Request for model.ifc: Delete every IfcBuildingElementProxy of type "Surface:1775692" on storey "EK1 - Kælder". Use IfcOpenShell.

First a look at what the model holds.

```python
import ifcopenshell
import ifcopenshell.util.element

model = ifcopenshell.open("model.ifc")
print(model.schema)
storey = next(s for s in model.by_type("IfcBuildingStorey") if s.Name == "EK1 - Kælder")
proxies = [e for e in ifcopenshell.util.element.get_decomposition(storey) if e.is_a("IfcBuildingElementProxy")]
seen = {}
for e in proxies:
    element_type = ifcopenshell.util.element.get_type(e)
    name = element_type.Name if element_type not in (None, e) else None
    seen[name] = seen.get(name, 0) + 1
for name, count in sorted(seen.items(), key=str):
    print(count, "x", name)
```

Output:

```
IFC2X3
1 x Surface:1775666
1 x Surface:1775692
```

```python
import ifcopenshell
import ifcopenshell.api.root
import ifcopenshell.util.element

model = ifcopenshell.open("model.ifc")

storey = next(s for s in model.by_type("IfcBuildingStorey") if s.Name == "EK1 - Kælder")
proxies = [e for e in ifcopenshell.util.element.get_decomposition(storey) if e.is_a("IfcBuildingElementProxy")]
targets = [e for e in proxies if (t := ifcopenshell.util.element.get_type(e)) not in (None, e) and t.Name == "Surface:1775692"]

for e in targets:
    ifcopenshell.api.root.remove_product(model, product=e)
print(len(targets), "removed")

model.write("model_rev.ifc")
```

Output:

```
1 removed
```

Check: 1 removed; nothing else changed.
